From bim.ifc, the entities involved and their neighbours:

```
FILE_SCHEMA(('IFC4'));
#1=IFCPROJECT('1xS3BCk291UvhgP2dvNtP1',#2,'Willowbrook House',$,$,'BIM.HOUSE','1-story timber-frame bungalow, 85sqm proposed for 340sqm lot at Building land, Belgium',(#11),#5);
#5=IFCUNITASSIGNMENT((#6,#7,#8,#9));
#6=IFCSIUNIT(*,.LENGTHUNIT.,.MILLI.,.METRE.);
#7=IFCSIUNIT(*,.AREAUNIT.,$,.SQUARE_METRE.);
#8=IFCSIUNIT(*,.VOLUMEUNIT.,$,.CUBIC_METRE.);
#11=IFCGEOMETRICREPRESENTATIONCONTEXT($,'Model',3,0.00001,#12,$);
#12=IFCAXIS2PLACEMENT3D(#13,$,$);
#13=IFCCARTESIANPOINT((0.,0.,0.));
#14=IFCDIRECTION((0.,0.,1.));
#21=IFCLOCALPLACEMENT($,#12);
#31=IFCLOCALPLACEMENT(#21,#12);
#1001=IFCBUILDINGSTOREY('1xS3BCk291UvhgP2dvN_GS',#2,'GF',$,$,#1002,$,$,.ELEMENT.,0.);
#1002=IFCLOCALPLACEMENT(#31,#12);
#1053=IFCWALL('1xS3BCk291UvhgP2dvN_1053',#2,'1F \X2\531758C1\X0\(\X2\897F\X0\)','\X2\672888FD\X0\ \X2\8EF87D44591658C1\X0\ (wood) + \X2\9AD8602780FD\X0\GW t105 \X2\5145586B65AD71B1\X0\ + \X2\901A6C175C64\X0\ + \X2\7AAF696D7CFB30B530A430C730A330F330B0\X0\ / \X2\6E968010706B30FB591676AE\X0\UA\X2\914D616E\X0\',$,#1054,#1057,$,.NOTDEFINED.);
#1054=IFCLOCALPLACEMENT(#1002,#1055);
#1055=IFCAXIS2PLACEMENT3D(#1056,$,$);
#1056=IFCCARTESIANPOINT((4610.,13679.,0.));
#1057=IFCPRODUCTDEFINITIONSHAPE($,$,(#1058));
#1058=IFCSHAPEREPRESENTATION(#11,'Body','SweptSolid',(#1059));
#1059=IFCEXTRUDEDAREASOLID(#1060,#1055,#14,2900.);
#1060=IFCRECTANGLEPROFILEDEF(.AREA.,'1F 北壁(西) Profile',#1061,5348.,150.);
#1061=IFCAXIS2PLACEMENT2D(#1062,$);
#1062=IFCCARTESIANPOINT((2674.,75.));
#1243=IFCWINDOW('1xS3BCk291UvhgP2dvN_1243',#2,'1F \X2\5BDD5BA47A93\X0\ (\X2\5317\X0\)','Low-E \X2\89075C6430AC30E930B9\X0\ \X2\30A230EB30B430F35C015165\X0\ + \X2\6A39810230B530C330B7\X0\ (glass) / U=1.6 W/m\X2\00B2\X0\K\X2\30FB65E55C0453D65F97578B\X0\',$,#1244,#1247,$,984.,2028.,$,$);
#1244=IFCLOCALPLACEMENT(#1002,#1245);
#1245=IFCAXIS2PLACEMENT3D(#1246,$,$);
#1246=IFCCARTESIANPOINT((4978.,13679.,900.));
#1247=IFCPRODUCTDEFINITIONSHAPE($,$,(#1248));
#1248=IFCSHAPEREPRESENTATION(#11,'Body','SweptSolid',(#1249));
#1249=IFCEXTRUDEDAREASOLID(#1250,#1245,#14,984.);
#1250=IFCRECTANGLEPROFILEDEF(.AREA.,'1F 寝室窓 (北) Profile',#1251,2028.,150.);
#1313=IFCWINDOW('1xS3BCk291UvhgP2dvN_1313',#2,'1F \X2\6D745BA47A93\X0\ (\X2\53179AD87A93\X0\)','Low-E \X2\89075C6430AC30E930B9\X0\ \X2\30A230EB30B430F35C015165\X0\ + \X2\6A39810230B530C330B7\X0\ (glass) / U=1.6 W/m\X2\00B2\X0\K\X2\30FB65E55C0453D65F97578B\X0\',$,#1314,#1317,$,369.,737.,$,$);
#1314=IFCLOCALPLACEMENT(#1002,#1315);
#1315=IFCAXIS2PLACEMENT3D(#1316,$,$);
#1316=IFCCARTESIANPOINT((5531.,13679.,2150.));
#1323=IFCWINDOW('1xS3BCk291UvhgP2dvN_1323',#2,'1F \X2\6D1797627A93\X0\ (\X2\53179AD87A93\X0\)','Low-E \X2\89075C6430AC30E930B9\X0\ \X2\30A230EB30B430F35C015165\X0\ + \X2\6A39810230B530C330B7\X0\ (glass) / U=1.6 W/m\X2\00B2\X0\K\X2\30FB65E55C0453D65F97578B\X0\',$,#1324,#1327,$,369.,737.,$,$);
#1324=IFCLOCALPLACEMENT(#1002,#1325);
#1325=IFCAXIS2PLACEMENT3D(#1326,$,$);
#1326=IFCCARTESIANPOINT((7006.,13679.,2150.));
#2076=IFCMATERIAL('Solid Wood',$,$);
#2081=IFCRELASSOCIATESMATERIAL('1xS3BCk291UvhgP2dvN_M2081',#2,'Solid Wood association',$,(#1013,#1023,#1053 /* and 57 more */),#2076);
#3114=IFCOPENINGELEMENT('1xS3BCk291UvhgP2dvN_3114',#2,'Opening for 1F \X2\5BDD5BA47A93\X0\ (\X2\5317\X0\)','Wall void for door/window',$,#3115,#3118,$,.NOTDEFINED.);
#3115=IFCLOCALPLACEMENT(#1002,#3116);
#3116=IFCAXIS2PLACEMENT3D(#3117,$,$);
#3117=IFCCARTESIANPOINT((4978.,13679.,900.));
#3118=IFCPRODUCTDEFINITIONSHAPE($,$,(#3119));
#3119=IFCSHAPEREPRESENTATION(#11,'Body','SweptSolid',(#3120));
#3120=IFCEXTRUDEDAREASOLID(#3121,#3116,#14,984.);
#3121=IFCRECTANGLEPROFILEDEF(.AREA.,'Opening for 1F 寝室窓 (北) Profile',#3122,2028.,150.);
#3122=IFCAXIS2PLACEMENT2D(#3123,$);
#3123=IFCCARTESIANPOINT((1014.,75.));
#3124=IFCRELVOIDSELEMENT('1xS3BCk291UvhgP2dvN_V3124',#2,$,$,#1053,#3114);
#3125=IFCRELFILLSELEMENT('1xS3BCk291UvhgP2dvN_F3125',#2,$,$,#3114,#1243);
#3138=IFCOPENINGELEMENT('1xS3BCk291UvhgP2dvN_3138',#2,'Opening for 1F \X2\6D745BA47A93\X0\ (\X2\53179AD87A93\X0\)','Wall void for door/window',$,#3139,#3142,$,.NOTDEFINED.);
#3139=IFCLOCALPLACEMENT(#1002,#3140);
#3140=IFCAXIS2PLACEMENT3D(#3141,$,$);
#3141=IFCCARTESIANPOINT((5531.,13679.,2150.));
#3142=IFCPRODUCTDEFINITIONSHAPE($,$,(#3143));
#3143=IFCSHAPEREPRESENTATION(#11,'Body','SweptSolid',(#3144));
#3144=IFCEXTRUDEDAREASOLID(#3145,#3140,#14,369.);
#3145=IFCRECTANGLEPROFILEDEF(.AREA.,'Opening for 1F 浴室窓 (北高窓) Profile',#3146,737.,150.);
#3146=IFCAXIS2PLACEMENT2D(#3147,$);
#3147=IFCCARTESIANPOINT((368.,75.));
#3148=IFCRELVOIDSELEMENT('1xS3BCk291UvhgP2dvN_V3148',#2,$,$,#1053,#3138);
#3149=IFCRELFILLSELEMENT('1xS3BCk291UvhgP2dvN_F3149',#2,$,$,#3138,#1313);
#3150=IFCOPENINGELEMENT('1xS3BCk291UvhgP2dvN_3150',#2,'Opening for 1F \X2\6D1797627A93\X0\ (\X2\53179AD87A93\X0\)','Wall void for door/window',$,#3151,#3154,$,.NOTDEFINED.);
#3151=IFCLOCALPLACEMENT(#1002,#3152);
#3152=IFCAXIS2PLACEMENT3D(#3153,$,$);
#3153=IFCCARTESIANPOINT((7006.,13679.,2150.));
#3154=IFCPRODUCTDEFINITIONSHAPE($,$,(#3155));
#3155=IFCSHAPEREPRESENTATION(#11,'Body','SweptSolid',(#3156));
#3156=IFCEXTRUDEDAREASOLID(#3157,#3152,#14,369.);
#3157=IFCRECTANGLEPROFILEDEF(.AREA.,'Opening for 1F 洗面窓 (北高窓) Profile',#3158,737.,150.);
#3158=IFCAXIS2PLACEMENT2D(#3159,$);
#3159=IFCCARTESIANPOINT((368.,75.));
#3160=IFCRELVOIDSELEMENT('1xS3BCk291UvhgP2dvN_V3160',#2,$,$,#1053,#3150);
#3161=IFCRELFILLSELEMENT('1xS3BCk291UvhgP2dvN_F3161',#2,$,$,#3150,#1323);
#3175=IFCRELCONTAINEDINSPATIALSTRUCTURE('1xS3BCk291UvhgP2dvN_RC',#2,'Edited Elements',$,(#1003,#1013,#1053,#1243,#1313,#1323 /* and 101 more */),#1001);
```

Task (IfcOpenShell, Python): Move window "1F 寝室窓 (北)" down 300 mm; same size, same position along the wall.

```python
import numpy as np
import ifcopenshell
import ifcopenshell.api.geometry
import ifcopenshell.util.placement
import ifcopenshell.util.unit

model = ifcopenshell.open("bim.ifc")
unit_scale = ifcopenshell.util.unit.calculate_unit_scale(model)

window = model.by_guid("1xS3BCk291UvhgP2dvN_1243")
opening = window.FillsVoids[0].RelatingOpeningElement
dz = -300.0

shift = np.array([0.0, 0.0, dz])
# The window is not placed relative to its opening, so move both.
for product in (opening, window):
    matrix = ifcopenshell.util.placement.get_local_placement(product.ObjectPlacement)
    matrix[:3, 3] += shift
    ifcopenshell.api.geometry.edit_object_placement(model, product=product, matrix=matrix, is_si=False)

print(f"moved by {dz * unit_scale:+.3f} m")

model.write("bim_updated.ifc")
```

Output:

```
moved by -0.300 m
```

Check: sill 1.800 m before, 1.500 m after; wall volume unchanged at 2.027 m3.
